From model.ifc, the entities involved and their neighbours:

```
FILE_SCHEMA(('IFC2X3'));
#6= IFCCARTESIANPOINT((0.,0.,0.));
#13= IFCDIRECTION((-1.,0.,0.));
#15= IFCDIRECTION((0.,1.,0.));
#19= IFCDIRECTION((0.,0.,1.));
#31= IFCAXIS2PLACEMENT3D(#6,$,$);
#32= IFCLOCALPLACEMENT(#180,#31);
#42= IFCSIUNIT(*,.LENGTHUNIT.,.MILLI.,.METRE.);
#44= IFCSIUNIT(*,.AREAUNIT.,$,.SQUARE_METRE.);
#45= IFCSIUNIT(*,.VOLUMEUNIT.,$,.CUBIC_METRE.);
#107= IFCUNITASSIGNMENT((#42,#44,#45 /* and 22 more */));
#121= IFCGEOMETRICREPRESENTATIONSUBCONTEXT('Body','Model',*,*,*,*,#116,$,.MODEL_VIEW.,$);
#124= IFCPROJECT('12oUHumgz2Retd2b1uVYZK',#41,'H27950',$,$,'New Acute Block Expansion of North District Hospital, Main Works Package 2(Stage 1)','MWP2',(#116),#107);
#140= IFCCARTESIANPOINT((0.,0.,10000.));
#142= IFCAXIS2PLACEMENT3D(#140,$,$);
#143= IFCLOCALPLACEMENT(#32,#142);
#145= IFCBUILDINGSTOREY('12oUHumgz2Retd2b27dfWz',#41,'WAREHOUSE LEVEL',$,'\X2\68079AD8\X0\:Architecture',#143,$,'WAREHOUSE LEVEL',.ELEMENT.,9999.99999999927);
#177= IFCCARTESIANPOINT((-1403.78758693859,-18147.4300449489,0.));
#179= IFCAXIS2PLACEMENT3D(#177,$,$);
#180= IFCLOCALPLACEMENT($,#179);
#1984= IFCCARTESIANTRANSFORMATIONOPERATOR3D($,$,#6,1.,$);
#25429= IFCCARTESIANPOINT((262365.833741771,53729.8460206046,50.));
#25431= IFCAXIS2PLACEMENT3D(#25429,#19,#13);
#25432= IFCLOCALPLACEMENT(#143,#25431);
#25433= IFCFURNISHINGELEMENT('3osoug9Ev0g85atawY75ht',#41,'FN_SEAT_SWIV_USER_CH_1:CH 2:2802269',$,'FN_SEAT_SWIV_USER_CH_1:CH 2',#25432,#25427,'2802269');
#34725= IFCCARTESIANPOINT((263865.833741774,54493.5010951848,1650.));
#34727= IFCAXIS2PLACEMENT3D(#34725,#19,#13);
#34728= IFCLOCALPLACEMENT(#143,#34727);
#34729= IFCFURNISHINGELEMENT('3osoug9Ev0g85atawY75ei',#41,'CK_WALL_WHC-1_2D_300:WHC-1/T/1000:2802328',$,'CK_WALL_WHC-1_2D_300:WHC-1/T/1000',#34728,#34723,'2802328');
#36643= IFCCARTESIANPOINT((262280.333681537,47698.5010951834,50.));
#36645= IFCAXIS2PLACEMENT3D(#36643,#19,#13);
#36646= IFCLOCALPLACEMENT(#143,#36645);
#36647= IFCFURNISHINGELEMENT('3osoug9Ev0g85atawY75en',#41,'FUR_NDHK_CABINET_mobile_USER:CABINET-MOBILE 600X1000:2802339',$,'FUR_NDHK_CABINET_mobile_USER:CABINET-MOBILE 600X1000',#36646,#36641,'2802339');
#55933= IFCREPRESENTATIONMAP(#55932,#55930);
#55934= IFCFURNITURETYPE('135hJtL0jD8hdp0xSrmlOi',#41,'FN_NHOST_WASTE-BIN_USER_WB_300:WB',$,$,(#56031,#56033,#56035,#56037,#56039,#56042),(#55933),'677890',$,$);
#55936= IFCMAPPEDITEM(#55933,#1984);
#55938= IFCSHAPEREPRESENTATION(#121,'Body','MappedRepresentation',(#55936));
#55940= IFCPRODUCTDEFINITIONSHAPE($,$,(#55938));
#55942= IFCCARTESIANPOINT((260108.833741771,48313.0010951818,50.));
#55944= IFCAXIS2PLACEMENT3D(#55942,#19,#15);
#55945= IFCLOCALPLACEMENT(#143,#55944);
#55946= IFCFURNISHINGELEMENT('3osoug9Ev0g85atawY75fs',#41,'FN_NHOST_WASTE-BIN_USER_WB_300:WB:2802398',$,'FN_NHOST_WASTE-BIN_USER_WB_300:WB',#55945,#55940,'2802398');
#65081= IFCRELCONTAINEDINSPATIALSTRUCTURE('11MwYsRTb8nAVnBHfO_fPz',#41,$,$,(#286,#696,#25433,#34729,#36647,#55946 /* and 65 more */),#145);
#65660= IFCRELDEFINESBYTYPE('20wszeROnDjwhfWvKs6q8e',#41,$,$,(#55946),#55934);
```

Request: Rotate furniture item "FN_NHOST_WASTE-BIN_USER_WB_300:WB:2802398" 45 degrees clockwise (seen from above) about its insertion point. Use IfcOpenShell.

```python
import ifcopenshell
import ifcopenshell.api.geometry
import ifcopenshell.util.placement

model = ifcopenshell.open("model.ifc")

item = model.by_guid("3osoug9Ev0g85atawY75fs")
matrix = ifcopenshell.util.placement.get_local_placement(item.ObjectPlacement)
matrix = matrix @ ifcopenshell.util.placement.rotation(-45, "Z")
ifcopenshell.api.geometry.edit_object_placement(model, product=item, matrix=matrix, is_si=False)

print(ifcopenshell.util.placement.get_local_placement(item.ObjectPlacement).round(3) + 0.0)

model.write("model_updated.ifc")
```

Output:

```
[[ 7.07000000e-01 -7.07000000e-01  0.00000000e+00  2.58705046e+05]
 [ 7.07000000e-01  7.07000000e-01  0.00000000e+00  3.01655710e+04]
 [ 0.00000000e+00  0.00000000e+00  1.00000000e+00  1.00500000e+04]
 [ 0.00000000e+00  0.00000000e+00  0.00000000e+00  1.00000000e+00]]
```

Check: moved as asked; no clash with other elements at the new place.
